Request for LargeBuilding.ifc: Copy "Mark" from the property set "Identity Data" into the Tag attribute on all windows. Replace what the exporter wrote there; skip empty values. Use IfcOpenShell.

First a look at what the model holds.

```python
import ifcopenshell
import ifcopenshell.util.element

model = ifcopenshell.open("LargeBuilding.ifc")
print(model.schema)
windows = model.by_type("IfcWindow")
print(len(windows), "windows")
for e in windows[:8]:
    source = ifcopenshell.util.element.get_pset(e, "Identity Data", "Mark")
    target = e.Tag
    print(e.id(), repr(source), repr(target), sep=" | ")
```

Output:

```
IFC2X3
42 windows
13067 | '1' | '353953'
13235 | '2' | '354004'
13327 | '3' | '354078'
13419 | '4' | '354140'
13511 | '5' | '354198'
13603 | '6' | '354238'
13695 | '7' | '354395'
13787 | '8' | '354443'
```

```python
import ifcopenshell
import ifcopenshell.util.element

model = ifcopenshell.open("LargeBuilding.ifc")

count = 0
for e in model.by_type("IfcWindow"):
    value = ifcopenshell.util.element.get_pset(e, "Identity Data", "Mark")
    current = e.Tag
    if not value or not value.strip() or current == value:
        continue
    e.Tag = value
    count += 1

print(count, "windows updated")

model.write("LargeBuilding_v2.ifc")
```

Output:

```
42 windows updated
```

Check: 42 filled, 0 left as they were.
